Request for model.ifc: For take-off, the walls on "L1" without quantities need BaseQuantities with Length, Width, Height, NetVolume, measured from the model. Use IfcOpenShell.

First a look at what the model holds.

```python
import ifcopenshell
import ifcopenshell.util.element
import ifcopenshell.util.unit

model = ifcopenshell.open("model.ifc")
print(model.schema)
for unit_type in ("LENGTHUNIT", "AREAUNIT", "VOLUMEUNIT"):
    print(unit_type, ifcopenshell.util.unit.calculate_unit_scale(model, unit_type))
storey = next(s for s in model.by_type("IfcBuildingStorey") if s.Name == "L1")
walls = [e for e in ifcopenshell.util.element.get_decomposition(storey) if e.is_a("IfcWall")]
for e in sorted(walls, key=lambda e: e.id()):
    print(e.id(), e.is_a(), e.Name, list(ifcopenshell.util.element.get_psets(e, qtos_only=True)), sep=" | ")
```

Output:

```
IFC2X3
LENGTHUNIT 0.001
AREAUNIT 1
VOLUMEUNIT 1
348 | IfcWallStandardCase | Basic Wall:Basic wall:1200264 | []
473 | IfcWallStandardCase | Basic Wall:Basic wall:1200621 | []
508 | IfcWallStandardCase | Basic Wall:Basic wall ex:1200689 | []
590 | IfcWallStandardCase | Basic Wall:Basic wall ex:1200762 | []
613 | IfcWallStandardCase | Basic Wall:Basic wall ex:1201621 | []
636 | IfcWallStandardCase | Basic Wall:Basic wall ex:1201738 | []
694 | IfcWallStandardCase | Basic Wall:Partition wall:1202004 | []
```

```python
import ifcopenshell
import ifcopenshell.api.pset
import ifcopenshell.geom
import ifcopenshell.util.element
import ifcopenshell.util.shape
import ifcopenshell.util.unit

model = ifcopenshell.open("model.ifc")
unit_scale = ifcopenshell.util.unit.calculate_unit_scale(model)
volume_scale = ifcopenshell.util.unit.calculate_unit_scale(model, "VOLUMEUNIT")
settings = ifcopenshell.geom.settings()

storey = next(s for s in model.by_type("IfcBuildingStorey") if s.Name == "L1")
walls = [e for e in ifcopenshell.util.element.get_decomposition(storey) if e.is_a("IfcWall")]

for e in sorted(walls, key=lambda e: e.id()):
    if ifcopenshell.util.element.get_psets(e, qtos_only=True, should_inherit=False):
        continue
    # Geometry comes back in metres, in the element's own axes.
    shape = ifcopenshell.geom.create_shape(settings, e)
    values = {
        "Length": ifcopenshell.util.shape.get_x(shape.geometry) / unit_scale,
        "Width": ifcopenshell.util.shape.get_y(shape.geometry) / unit_scale,
        "Height": ifcopenshell.util.shape.get_z(shape.geometry) / unit_scale,
        "NetVolume": ifcopenshell.util.shape.get_volume(shape.geometry) / volume_scale,
    }
    qto = ifcopenshell.api.pset.add_qto(model, product=e, name="BaseQuantities")
    ifcopenshell.api.pset.edit_qto(model, qto=qto, properties=values)
    print(e.id(), {k: round(v, 3) for k, v in values.items()})

model.write("model_v2.ifc")
```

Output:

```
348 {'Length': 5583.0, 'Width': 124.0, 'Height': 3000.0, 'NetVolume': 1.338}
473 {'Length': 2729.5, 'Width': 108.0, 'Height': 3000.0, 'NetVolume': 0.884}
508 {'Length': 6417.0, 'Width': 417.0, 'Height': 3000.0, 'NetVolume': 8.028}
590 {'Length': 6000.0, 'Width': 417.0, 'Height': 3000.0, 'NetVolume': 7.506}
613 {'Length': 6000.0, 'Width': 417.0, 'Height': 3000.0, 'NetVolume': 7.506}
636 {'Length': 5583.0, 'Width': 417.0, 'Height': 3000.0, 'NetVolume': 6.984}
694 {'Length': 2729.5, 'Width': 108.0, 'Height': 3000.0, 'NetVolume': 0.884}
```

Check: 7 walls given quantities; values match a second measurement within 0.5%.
